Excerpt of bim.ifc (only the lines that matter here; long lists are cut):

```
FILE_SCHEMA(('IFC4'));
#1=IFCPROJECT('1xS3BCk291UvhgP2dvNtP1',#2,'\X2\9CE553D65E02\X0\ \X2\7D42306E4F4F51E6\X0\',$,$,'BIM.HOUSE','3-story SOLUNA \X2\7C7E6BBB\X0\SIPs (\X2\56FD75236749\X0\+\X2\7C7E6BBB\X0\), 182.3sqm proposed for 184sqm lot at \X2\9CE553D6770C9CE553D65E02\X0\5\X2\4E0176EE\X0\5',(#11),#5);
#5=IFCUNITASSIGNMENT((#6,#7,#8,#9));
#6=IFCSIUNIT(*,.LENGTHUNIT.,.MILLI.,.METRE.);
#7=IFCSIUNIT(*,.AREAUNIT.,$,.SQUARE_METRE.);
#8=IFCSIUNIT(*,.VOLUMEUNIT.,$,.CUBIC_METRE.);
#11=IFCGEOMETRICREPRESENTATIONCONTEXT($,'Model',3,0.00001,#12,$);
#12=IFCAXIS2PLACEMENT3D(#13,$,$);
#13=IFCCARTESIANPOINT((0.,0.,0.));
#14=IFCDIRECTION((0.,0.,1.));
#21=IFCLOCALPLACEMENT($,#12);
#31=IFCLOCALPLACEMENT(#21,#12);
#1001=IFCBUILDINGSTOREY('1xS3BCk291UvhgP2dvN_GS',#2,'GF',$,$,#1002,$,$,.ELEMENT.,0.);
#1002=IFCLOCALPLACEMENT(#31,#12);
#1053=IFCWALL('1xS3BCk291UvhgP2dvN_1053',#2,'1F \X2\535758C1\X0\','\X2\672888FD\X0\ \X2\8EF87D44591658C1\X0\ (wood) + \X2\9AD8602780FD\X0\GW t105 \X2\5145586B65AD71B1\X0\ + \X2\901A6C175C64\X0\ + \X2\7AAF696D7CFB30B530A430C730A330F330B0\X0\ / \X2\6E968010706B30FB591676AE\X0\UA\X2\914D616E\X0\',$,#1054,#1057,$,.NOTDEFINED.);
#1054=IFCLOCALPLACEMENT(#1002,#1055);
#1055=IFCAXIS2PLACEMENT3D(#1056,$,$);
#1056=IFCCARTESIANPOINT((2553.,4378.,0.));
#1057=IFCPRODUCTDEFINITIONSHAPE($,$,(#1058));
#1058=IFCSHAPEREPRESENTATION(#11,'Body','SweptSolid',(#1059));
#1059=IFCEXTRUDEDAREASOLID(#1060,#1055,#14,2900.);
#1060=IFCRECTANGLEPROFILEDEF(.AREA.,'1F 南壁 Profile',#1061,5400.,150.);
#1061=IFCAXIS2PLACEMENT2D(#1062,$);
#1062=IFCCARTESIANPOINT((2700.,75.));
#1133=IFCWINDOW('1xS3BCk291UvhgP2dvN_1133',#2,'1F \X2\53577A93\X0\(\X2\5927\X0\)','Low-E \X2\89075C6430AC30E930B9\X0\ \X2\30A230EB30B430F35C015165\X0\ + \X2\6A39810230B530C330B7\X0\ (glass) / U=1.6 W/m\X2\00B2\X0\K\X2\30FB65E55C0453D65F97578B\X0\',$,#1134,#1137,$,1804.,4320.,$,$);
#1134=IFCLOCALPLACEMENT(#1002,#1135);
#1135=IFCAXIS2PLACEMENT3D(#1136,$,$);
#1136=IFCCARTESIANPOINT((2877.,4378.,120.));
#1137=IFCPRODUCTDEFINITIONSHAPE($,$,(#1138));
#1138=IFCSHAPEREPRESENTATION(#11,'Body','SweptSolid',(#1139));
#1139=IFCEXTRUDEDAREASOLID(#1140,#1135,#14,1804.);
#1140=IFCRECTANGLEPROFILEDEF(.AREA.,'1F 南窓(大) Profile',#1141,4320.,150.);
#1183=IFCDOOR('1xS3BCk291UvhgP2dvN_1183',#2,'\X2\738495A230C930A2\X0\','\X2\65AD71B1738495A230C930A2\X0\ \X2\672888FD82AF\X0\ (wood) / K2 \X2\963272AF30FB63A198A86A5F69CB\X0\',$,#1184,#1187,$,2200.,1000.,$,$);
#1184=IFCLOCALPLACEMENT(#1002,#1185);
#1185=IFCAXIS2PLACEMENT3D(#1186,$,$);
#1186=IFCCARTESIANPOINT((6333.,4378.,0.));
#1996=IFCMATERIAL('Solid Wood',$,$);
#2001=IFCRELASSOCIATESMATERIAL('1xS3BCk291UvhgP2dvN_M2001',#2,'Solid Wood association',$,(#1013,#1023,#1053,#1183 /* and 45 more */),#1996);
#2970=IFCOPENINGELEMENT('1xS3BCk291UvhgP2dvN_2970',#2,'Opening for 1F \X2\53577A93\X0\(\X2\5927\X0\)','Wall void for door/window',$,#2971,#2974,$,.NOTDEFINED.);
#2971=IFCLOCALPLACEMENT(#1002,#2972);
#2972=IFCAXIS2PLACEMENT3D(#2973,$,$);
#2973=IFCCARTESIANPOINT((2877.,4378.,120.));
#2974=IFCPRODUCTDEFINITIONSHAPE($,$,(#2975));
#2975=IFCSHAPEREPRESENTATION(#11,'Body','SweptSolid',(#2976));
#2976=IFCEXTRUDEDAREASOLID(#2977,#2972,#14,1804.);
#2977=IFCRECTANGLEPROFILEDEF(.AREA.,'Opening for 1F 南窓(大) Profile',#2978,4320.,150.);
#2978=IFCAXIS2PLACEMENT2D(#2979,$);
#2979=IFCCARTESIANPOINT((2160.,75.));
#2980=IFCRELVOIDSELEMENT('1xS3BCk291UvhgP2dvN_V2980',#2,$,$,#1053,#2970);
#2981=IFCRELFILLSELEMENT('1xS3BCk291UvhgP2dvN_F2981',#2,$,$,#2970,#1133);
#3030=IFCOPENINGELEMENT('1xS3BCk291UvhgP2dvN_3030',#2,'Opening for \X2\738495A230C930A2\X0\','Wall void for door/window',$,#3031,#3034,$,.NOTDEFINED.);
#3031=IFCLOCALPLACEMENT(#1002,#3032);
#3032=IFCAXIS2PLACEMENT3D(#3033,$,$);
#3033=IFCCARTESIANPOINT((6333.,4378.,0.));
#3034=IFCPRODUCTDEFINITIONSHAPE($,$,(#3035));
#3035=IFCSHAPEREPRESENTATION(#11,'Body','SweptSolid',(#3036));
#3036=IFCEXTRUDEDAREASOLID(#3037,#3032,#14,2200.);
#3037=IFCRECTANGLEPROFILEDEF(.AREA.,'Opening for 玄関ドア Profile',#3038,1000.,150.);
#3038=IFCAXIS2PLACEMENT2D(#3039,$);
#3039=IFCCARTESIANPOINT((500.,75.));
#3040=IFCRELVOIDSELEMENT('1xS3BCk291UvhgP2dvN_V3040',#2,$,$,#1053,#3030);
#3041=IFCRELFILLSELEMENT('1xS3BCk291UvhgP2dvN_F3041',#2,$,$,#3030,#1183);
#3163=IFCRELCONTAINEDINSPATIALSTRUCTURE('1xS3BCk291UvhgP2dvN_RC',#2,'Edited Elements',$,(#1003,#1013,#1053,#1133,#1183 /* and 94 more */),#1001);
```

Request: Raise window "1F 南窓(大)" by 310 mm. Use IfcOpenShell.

```python
import numpy as np
import ifcopenshell
import ifcopenshell.api.geometry
import ifcopenshell.util.placement
import ifcopenshell.util.unit

model = ifcopenshell.open("bim.ifc")
unit_scale = ifcopenshell.util.unit.calculate_unit_scale(model)

window = model.by_guid("1xS3BCk291UvhgP2dvN_1133")
opening = window.FillsVoids[0].RelatingOpeningElement
dz = 0.31 / unit_scale

shift = np.array([0.0, 0.0, dz])
# The window is not placed relative to its opening, so move both.
for product in (opening, window):
    matrix = ifcopenshell.util.placement.get_local_placement(product.ObjectPlacement)
    matrix[:3, 3] += shift
    ifcopenshell.api.geometry.edit_object_placement(model, product=product, matrix=matrix, is_si=False)

print(f"moved by {dz * unit_scale:+.3f} m")

model.write("bim-out.ifc")
```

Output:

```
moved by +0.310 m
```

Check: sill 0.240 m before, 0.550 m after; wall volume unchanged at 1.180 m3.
